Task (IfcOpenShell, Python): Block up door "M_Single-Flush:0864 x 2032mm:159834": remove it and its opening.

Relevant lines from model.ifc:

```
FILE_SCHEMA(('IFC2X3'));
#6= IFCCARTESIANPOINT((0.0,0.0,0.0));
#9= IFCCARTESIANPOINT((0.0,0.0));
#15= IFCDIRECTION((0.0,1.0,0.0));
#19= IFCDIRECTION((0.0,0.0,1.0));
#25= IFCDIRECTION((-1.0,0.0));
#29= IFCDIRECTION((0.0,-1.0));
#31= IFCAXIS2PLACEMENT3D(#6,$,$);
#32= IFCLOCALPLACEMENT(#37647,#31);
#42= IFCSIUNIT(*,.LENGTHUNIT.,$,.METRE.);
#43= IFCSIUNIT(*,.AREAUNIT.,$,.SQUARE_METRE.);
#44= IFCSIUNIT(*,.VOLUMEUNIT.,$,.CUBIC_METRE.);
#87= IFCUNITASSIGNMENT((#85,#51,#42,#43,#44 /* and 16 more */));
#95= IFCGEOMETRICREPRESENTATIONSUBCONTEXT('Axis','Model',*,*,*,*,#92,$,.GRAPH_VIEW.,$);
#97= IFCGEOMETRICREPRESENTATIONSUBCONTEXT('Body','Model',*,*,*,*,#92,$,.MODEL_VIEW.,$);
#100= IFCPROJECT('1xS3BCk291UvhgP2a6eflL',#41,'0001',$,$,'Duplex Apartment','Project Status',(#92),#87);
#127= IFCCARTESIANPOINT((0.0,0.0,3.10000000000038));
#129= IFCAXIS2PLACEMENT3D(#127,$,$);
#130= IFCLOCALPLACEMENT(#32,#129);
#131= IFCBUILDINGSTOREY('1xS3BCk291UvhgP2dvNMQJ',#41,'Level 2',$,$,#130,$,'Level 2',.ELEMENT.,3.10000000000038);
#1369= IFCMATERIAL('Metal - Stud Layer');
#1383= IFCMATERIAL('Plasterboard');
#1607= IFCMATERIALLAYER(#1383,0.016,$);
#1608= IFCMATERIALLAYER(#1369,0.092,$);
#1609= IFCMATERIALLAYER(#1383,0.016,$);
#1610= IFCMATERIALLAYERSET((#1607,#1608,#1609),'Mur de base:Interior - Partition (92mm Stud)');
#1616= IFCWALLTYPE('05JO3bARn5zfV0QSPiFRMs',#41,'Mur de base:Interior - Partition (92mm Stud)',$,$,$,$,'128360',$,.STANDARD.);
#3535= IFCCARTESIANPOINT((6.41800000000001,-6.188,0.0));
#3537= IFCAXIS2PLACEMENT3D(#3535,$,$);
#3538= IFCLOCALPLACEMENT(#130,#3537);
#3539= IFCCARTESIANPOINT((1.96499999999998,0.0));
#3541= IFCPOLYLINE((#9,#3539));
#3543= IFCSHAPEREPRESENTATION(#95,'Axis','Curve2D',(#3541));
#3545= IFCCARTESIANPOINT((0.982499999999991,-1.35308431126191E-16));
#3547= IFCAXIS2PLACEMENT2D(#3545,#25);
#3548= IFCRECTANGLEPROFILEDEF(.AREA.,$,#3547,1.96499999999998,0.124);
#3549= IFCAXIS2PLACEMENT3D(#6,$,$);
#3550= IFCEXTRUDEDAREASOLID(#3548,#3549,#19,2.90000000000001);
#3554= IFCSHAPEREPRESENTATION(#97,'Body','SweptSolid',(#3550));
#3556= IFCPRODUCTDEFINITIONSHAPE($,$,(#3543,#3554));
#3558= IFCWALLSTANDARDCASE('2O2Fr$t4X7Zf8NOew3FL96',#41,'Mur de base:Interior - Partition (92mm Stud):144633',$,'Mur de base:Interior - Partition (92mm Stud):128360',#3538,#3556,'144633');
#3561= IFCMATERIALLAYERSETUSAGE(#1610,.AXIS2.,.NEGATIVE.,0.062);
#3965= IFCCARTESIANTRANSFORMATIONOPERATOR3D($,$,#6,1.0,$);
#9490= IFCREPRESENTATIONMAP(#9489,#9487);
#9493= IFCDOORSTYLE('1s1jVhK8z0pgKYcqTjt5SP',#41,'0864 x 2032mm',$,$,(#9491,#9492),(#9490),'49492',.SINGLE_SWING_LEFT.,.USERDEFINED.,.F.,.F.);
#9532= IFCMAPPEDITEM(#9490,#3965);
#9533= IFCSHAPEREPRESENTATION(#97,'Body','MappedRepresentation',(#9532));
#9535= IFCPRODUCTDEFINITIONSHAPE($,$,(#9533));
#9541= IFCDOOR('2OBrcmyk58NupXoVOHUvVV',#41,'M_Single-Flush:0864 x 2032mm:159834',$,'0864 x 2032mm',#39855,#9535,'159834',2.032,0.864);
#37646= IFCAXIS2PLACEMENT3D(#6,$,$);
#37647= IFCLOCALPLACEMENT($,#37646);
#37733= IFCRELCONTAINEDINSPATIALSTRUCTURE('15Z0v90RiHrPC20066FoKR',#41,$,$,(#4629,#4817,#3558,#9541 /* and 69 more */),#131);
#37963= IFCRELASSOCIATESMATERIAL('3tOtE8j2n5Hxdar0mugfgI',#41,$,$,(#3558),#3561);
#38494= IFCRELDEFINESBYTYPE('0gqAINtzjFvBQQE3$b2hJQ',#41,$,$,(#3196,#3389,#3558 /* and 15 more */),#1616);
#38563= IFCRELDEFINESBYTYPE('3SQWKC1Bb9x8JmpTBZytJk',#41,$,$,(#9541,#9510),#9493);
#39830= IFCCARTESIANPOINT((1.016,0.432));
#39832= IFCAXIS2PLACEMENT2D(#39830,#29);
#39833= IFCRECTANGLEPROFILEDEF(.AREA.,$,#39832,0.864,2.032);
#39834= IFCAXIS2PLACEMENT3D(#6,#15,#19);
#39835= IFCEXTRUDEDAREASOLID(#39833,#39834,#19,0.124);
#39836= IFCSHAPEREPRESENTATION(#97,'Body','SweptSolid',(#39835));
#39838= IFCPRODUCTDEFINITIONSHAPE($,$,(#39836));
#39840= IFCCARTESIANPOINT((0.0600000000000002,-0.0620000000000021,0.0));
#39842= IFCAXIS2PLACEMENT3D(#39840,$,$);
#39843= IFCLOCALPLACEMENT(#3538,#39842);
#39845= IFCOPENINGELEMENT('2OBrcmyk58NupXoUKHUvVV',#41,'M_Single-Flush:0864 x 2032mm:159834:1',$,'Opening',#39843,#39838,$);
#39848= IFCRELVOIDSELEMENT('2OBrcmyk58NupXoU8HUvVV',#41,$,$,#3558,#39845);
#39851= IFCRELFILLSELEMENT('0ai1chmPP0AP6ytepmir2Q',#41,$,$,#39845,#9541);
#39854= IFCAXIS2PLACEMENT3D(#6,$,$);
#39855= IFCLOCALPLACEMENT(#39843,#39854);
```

```python
import ifcopenshell
import ifcopenshell.api.feature
import ifcopenshell.api.root
import ifcopenshell.geom
import ifcopenshell.util.shape

model = ifcopenshell.open("model.ifc")
settings = ifcopenshell.geom.settings()


def volume(element):
    """Net volume in cubic metres, openings subtracted."""
    shape = ifcopenshell.geom.create_shape(settings, element)
    return ifcopenshell.util.shape.get_volume(shape.geometry)


door = model.by_guid("2OBrcmyk58NupXoVOHUvVV")
opening = door.FillsVoids[0].RelatingOpeningElement
wall = opening.VoidsElements[0].RelatingBuildingElement
before = volume(wall)

ifcopenshell.api.root.remove_product(model, product=door)
ifcopenshell.api.feature.remove_feature(model, feature=opening)

after = volume(wall)

print(f"wall volume {before:.3f} -> {after:.3f} m3")

model.write("model-out.ifc")
```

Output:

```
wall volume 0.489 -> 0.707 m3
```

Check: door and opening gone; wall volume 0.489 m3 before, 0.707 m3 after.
